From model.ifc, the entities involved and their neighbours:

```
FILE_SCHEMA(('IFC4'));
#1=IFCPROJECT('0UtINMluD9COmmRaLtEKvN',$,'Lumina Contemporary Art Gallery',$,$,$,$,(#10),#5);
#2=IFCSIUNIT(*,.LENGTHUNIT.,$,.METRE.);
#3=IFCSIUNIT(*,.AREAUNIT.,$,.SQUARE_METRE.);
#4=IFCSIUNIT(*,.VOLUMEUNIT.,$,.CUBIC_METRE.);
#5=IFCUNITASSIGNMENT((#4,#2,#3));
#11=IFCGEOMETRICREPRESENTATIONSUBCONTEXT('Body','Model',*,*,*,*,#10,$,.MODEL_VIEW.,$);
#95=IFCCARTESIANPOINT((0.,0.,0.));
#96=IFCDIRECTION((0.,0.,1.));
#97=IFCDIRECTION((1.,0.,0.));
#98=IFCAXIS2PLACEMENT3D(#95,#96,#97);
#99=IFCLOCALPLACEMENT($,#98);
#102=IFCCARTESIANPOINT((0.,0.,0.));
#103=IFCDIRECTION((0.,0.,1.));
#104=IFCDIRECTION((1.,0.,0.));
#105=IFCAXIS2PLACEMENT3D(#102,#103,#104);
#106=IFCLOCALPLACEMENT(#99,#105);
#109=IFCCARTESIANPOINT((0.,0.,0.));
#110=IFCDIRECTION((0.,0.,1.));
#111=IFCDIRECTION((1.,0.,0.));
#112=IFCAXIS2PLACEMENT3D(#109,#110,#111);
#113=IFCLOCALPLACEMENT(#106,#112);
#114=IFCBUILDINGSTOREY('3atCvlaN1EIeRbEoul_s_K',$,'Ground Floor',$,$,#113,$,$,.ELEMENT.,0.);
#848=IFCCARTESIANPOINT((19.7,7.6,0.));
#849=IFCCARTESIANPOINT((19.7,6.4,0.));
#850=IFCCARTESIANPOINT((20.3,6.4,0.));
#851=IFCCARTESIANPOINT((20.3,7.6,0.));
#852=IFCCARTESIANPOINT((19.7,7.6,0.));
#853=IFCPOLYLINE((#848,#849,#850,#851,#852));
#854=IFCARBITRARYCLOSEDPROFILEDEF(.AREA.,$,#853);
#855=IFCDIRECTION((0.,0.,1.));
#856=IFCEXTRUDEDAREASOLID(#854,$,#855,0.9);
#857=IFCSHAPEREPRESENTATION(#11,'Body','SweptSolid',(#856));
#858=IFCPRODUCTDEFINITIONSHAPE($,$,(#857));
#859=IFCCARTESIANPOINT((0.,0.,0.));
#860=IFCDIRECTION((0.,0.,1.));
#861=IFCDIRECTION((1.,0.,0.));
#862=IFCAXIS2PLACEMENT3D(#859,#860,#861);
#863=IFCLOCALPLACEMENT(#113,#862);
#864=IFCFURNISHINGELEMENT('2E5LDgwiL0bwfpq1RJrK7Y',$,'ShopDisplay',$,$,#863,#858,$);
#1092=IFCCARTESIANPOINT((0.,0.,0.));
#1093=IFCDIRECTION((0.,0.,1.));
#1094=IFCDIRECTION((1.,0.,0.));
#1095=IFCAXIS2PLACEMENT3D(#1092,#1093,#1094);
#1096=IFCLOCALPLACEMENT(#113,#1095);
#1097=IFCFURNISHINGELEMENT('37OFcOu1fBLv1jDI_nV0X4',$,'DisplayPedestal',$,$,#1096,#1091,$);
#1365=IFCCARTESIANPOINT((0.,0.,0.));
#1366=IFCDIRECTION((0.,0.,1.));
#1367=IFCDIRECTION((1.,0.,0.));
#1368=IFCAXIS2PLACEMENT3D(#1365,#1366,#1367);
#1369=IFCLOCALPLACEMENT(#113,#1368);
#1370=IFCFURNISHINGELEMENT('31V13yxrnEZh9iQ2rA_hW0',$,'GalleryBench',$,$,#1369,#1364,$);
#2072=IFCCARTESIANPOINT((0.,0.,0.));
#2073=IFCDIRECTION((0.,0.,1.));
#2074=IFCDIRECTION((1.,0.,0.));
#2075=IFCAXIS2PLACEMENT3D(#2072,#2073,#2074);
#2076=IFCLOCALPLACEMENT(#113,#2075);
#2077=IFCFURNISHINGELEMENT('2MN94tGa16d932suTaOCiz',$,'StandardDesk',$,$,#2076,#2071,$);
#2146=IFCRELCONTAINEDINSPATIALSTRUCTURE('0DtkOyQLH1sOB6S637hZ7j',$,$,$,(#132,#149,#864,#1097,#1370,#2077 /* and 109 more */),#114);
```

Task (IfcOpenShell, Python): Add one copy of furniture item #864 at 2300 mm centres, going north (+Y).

```python
import numpy as np
import ifcopenshell
import ifcopenshell.api.geometry
import ifcopenshell.api.root
import ifcopenshell.util.element
import ifcopenshell.util.placement

model = ifcopenshell.open("model.ifc")

source = model.by_id(864)
base = ifcopenshell.util.placement.get_local_placement(source.ObjectPlacement)
step = np.array([0.0, 1.0, 0.0]) * 2.3

for i in range(1, 2):
    copy = ifcopenshell.api.root.copy_class(model, product=source)
    copy.Representation = ifcopenshell.util.element.copy_deep(
        model, source.Representation, exclude=["IfcGeometricRepresentationContext", "IfcRepresentationMap"]
    )
    matrix = base.copy()
    matrix[:3, 3] += i * step
    print("added at", matrix[:3, 3].round(3) + 0.0)
    ifcopenshell.api.geometry.edit_object_placement(model, product=copy, matrix=matrix, is_si=False)

model.write("model-out.ifc")
```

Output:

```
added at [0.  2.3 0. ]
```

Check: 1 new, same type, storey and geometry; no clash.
